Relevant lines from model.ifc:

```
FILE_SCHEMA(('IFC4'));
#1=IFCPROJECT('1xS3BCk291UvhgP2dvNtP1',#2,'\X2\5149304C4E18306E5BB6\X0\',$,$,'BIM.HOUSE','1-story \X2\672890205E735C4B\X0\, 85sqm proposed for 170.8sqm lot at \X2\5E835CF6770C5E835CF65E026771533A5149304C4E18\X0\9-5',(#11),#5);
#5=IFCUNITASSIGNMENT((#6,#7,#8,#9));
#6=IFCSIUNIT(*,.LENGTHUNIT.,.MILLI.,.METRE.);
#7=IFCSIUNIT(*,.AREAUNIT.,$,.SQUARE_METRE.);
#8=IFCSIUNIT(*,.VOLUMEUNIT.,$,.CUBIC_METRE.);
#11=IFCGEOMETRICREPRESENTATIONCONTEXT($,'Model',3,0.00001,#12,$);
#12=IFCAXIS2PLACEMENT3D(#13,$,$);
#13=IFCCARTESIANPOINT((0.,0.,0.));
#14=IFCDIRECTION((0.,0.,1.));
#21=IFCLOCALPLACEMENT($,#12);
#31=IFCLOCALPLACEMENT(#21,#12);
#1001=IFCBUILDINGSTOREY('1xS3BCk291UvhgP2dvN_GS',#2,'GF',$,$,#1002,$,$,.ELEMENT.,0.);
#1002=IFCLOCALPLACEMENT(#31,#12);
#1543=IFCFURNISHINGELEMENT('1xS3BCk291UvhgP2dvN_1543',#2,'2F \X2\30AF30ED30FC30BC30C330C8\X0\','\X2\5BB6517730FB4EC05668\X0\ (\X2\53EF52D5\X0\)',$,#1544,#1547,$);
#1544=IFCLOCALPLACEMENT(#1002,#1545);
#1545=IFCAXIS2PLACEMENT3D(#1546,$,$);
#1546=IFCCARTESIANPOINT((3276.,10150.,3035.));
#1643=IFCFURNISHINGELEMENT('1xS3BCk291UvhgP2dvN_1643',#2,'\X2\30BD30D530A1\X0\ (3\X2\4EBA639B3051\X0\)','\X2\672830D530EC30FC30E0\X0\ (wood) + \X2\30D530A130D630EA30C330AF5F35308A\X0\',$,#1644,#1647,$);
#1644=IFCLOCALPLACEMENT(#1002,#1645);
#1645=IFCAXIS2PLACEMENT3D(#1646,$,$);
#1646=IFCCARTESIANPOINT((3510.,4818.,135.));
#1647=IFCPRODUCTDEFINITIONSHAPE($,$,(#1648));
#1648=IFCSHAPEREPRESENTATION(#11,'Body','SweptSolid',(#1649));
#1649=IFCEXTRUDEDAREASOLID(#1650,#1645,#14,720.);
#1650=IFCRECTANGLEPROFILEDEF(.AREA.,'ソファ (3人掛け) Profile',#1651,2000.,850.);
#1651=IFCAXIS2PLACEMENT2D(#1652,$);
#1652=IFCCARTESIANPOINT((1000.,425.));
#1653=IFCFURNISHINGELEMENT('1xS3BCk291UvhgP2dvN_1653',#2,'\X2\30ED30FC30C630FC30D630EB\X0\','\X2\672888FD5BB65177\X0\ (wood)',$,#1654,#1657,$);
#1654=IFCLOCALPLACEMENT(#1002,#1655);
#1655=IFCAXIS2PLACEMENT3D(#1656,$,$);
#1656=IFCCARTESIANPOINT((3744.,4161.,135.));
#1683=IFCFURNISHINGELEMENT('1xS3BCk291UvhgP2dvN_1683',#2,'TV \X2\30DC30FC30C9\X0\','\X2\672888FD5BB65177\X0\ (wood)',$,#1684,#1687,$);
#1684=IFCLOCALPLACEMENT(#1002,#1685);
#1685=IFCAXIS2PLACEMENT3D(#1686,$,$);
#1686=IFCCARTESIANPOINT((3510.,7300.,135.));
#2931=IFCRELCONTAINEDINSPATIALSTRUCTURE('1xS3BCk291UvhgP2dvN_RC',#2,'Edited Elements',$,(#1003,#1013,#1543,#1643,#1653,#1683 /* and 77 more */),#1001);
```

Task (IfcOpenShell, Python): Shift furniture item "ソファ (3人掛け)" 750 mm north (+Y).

```python
import ifcopenshell
import ifcopenshell.api.geometry
import ifcopenshell.util.placement
import ifcopenshell.util.unit

model = ifcopenshell.open("model.ifc")
unit_scale = ifcopenshell.util.unit.calculate_unit_scale(model)

item = model.by_guid("1xS3BCk291UvhgP2dvN_1643")
matrix = ifcopenshell.util.placement.get_local_placement(item.ObjectPlacement)
matrix[1, 3] += 0.75 / unit_scale
ifcopenshell.api.geometry.edit_object_placement(model, product=item, matrix=matrix, is_si=False)

print(ifcopenshell.util.placement.get_local_placement(item.ObjectPlacement).round(3) + 0.0)

model.write("model_updated.ifc")
```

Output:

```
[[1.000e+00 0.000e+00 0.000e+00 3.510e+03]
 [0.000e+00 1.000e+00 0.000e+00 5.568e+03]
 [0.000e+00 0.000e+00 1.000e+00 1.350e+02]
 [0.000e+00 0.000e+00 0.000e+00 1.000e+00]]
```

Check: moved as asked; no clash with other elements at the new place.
